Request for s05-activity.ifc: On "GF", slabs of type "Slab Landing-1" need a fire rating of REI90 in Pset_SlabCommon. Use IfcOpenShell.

First a look at what the model holds.

```python
import ifcopenshell
import ifcopenshell.util.element

model = ifcopenshell.open("s05-activity.ifc")
print(model.schema)
storey = next(s for s in model.by_type("IfcBuildingStorey") if s.Name == "GF")
slabs = [e for e in ifcopenshell.util.element.get_decomposition(storey) if e.is_a("IfcSlab")]
seen = {}
for e in slabs:
    element_type = ifcopenshell.util.element.get_type(e)
    key = (element_type.Name if element_type != e and element_type else None, ifcopenshell.util.element.get_pset(e, "Pset_SlabCommon", "FireRating"))
    seen[key] = seen.get(key, 0) + 1
for (name, value), count in sorted(seen.items(), key=str):
    print(count, "x", name, "|", value)
```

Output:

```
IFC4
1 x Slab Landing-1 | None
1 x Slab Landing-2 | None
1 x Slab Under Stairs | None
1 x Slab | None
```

```python
import ifcopenshell
import ifcopenshell.api.pset
import ifcopenshell.util.element

model = ifcopenshell.open("s05-activity.ifc")

storey = next(s for s in model.by_type("IfcBuildingStorey") if s.Name == "GF")
slabs = [e for e in ifcopenshell.util.element.get_decomposition(storey) if e.is_a("IfcSlab")]

count = 0
for e in slabs:
    element_type = ifcopenshell.util.element.get_type(e)
    if element_type in (None, e) or element_type.Name != "Slab Landing-1":
        continue
    # add_pset returns the element's existing set when there is one.
    pset = ifcopenshell.api.pset.add_pset(model, product=e, name="Pset_SlabCommon")
    ifcopenshell.api.pset.edit_pset(model, pset=pset, properties={"FireRating": "REI90"})
    count += 1

print(count, "slabs updated")

model.write("s05-activity-out.ifc")
```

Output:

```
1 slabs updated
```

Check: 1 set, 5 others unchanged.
